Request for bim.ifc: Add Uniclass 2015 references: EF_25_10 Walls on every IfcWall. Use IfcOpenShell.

First a look at what the model holds.

```python
import ifcopenshell

model = ifcopenshell.open("bim.ifc")
print(model.schema)
print("classifications:", [c.Name for c in model.by_type("IfcClassification")])
for ifc_class in ("IfcDoor", "IfcRoof", "IfcStair", "IfcWall", "IfcWindow"):
    print(ifc_class, len(model.by_type(ifc_class)))
```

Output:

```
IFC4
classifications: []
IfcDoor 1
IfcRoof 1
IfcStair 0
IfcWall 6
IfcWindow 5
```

```python
import ifcopenshell
import ifcopenshell.api.classification

model = ifcopenshell.open("bim.ifc")

system = ifcopenshell.api.classification.add_classification(model, classification="Uniclass 2015")

codes = {
    "IfcWall": ("EF_25_10", "Walls"),
}
for ifc_class, (code, name) in codes.items():
    products = model.by_type(ifc_class)
    ifcopenshell.api.classification.add_reference(
        model, products=products, classification=system, identification=code, name=name
    )
    print(code, len(products))

model.write("bim-out.ifc")
```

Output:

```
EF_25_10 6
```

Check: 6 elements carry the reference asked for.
